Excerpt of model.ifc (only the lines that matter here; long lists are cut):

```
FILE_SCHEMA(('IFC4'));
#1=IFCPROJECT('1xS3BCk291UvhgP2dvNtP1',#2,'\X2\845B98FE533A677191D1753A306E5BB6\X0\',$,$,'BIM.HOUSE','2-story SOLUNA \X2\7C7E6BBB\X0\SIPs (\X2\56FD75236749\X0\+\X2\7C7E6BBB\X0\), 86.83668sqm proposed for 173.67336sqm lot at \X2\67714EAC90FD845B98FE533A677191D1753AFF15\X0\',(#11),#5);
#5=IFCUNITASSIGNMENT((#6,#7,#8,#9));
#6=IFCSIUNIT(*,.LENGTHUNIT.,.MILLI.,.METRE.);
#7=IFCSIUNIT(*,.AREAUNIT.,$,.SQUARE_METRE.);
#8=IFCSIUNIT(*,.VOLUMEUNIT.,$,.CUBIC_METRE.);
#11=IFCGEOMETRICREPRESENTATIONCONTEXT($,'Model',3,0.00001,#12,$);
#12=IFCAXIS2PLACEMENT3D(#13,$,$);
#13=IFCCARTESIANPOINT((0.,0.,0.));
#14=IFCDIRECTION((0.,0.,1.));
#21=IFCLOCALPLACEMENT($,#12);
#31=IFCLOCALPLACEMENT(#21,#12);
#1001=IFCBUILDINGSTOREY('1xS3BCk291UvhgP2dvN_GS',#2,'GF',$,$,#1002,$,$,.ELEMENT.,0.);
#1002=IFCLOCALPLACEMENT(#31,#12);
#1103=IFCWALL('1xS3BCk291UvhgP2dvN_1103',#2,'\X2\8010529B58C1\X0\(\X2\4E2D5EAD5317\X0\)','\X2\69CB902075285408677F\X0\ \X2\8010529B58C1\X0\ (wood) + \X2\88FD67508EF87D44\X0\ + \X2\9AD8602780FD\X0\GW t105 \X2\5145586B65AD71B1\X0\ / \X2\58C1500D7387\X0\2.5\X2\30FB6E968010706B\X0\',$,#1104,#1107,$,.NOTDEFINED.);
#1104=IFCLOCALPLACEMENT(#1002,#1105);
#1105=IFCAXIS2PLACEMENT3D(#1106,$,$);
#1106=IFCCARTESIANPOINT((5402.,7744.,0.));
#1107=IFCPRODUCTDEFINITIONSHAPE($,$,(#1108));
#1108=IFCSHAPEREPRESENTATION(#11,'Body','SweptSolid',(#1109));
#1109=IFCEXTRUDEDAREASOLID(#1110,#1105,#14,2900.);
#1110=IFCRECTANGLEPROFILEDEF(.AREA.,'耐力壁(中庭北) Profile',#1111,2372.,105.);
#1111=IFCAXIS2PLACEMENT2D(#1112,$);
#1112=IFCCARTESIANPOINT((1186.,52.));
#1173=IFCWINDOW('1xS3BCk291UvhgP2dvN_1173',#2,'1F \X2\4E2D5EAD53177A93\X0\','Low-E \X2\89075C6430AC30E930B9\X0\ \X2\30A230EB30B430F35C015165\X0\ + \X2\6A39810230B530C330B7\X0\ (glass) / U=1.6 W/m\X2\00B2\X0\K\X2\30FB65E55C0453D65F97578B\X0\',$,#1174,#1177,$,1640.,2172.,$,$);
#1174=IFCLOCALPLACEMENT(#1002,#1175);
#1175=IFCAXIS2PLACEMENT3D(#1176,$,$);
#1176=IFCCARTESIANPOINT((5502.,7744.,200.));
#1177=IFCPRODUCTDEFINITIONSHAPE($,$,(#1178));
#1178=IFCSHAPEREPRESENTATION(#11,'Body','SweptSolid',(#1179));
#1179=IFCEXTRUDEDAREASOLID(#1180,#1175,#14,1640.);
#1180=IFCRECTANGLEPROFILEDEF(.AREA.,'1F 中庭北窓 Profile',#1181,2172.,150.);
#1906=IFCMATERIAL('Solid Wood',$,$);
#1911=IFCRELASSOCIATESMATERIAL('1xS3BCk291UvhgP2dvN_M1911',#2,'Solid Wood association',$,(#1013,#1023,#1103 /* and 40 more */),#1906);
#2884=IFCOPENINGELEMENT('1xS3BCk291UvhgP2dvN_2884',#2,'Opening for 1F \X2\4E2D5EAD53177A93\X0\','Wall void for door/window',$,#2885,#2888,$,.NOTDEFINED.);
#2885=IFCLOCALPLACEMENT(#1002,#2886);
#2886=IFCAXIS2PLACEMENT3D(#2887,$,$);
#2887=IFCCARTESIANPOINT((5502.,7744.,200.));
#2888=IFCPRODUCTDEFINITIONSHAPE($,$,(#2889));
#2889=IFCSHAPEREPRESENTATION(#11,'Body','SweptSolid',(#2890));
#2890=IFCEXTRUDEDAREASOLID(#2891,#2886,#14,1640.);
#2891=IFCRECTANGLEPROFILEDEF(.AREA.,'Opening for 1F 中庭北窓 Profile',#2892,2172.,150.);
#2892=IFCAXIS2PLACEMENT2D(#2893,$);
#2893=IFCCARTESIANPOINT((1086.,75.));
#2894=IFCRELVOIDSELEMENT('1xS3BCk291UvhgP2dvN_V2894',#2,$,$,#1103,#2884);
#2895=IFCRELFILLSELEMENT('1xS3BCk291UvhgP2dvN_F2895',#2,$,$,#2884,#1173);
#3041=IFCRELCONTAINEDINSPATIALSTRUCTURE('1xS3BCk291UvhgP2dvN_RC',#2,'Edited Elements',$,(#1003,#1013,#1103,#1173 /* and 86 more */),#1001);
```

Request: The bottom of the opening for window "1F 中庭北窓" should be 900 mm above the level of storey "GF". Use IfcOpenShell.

```python
import numpy as np
import ifcopenshell
import ifcopenshell.api.geometry
import ifcopenshell.geom
import ifcopenshell.util.element
import ifcopenshell.util.placement
import ifcopenshell.util.shape
import ifcopenshell.util.unit

model = ifcopenshell.open("model.ifc")
unit_scale = ifcopenshell.util.unit.calculate_unit_scale(model)

window = model.by_guid("1xS3BCk291UvhgP2dvN_1173")
opening = window.FillsVoids[0].RelatingOpeningElement
storey = ifcopenshell.util.element.get_container(window, ifc_class="IfcBuildingStorey")
level = ifcopenshell.util.placement.get_local_placement(storey.ObjectPlacement)[2, 3]

# The opening's origin need not be at the sill, so measure its lowest point.
shape = ifcopenshell.geom.create_shape(ifcopenshell.geom.settings(), opening)
bottom = ifcopenshell.util.shape.get_shape_bottom_elevation(shape, shape.geometry) / unit_scale
dz = level + 900.0 - bottom

shift = np.array([0.0, 0.0, dz])
# The window is not placed relative to its opening, so move both.
for product in (opening, window):
    matrix = ifcopenshell.util.placement.get_local_placement(product.ObjectPlacement)
    matrix[:3, 3] += shift
    ifcopenshell.api.geometry.edit_object_placement(model, product=product, matrix=matrix, is_si=False)

print(f"moved by {dz * unit_scale:+.3f} m")

model.write("model_rev.ifc")
```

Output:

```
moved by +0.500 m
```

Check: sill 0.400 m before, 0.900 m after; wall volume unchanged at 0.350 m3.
